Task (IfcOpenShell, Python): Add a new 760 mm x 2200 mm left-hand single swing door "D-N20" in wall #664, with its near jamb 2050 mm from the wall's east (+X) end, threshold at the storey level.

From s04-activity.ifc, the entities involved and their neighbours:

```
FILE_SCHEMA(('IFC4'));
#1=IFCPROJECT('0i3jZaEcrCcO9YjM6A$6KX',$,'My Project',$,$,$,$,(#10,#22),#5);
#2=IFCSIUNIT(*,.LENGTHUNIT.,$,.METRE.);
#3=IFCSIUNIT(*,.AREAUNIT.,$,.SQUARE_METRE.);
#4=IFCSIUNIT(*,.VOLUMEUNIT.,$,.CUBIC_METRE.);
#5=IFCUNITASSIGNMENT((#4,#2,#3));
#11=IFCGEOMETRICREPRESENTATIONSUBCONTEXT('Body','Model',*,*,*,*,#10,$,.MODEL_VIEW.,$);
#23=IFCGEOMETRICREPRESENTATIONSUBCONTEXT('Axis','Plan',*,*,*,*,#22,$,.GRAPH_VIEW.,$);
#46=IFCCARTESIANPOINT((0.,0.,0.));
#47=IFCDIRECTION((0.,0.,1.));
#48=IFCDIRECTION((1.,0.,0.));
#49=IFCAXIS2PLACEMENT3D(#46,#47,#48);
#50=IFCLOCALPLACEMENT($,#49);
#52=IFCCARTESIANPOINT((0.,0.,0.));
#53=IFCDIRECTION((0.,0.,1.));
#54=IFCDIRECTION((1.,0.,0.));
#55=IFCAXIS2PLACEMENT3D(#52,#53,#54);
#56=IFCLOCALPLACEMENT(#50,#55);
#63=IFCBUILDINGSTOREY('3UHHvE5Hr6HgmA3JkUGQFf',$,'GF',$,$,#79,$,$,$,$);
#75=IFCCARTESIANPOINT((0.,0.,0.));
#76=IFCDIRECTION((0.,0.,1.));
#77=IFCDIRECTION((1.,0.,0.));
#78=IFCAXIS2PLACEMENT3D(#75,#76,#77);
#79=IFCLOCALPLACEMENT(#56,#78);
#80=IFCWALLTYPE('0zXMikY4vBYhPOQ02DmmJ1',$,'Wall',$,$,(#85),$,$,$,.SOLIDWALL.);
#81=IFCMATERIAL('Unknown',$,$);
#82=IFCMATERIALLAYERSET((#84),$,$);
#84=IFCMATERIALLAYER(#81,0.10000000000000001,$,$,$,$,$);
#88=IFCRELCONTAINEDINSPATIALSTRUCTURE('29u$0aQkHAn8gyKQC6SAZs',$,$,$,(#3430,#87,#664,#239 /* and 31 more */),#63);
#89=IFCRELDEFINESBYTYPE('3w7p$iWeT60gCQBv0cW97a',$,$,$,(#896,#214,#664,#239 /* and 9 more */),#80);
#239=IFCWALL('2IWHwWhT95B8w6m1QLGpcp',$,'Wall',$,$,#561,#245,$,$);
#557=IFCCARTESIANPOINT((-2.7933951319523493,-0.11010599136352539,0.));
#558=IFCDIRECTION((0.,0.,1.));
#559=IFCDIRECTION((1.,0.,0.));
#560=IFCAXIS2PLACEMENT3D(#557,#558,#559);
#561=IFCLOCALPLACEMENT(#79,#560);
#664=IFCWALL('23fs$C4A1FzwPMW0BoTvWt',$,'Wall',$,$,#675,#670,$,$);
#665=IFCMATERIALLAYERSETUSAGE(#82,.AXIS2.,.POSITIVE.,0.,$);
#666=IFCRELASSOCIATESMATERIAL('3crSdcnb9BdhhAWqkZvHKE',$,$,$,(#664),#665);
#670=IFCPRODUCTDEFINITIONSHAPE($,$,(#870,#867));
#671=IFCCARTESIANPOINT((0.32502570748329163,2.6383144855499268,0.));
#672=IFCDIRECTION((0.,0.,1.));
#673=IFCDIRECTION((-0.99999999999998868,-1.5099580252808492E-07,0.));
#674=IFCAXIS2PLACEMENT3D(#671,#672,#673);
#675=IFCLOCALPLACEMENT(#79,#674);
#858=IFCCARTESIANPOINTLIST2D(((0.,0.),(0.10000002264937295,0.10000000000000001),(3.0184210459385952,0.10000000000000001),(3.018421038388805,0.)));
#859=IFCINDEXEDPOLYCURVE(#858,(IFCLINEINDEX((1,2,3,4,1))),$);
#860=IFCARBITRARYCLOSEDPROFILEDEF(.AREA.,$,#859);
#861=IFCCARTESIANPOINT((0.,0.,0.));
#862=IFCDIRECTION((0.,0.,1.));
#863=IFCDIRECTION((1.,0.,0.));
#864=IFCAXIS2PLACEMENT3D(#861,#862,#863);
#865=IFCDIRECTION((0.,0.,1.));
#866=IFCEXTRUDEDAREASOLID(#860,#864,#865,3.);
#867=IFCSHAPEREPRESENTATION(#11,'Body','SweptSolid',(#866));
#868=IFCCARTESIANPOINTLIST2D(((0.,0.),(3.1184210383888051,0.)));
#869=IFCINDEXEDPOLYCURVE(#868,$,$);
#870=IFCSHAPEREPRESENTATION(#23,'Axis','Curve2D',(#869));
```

```python
import numpy as np
import ifcopenshell
import ifcopenshell.api.feature
import ifcopenshell.api.geometry
import ifcopenshell.api.root
import ifcopenshell.api.spatial
import ifcopenshell.geom
import ifcopenshell.util.element
import ifcopenshell.util.placement
import ifcopenshell.util.representation
import ifcopenshell.util.shape
import ifcopenshell.util.unit

model = ifcopenshell.open("s04-activity.ifc")
unit_scale = ifcopenshell.util.unit.calculate_unit_scale(model)
settings = ifcopenshell.geom.settings()


def volume(element):
    """Net volume in cubic metres, openings subtracted."""
    shape = ifcopenshell.geom.create_shape(settings, element)
    return ifcopenshell.util.shape.get_volume(shape.geometry)


wall = model.by_guid("23fs$C4A1FzwPMW0BoTvWt")
storey = ifcopenshell.util.element.get_container(wall, ifc_class="IfcBuildingStorey")
context = ifcopenshell.util.representation.get_context(model, "Model", "Body", "MODEL_VIEW")
before = volume(wall)

width, height, from_end, sill = 0.76, 2.2, 2.05, 0.0  # metres

# The wall runs along its own X axis, and the end named is its -X end.
wall_shape = ifcopenshell.geom.create_shape(settings, wall)
x, y, z = ifcopenshell.util.shape.get_vertices(wall_shape.geometry).T
start = x.min() + from_end
face, thickness = float(y.min()), float(y.max() - y.min())
wall_matrix = ifcopenshell.util.placement.get_local_placement(wall.ObjectPlacement)
level = ifcopenshell.util.placement.get_local_placement(storey.ObjectPlacement)[2, 3]


def in_wall(x, y):
    """Placement at x, y metres in the wall's axes, at sill height."""
    matrix = wall_matrix.copy()
    matrix[:, 3] = wall_matrix @ np.array([x / unit_scale, y / unit_scale, 0.0, 1.0])
    matrix[2, 3] = level + sill / unit_scale
    return matrix


# Opening: a box that overshoots both wall faces by 50 mm.
opening = ifcopenshell.api.root.create_entity(model, ifc_class="IfcOpeningElement", predefined_type="OPENING")
box = ifcopenshell.api.geometry.add_wall_representation(
    model, context=context, length=width, height=height, thickness=thickness + 0.1
)
ifcopenshell.api.geometry.assign_representation(model, product=opening, representation=box)
ifcopenshell.api.geometry.edit_object_placement(model, product=opening, matrix=in_wall(start, face - 0.05), is_si=False)
ifcopenshell.api.feature.add_feature(model, feature=opening, element=wall)

door = ifcopenshell.api.root.create_entity(model, ifc_class="IfcDoor", name="D-N20", predefined_type="DOOR")
door.OverallWidth, door.OverallHeight = width / unit_scale, height / unit_scale
door.OperationType = "SINGLE_SWING_LEFT"
body = ifcopenshell.api.geometry.add_door_representation(
    model,
    context=context,
    overall_width=door.OverallWidth,
    overall_height=door.OverallHeight,
    operation_type="SINGLE_SWING_LEFT",
    lining_properties={"LiningDepth": thickness / unit_scale, "ThresholdDepth": thickness / unit_scale},
)
ifcopenshell.api.geometry.assign_representation(model, product=door, representation=body)
ifcopenshell.api.spatial.assign_container(model, products=[door], relating_structure=storey)
ifcopenshell.api.feature.add_filling(model, opening=opening, element=door)

# The lining spans the wall, so the door starts at the wall face.
ifcopenshell.api.geometry.edit_object_placement(model, product=door, matrix=in_wall(start, face), is_si=False)

after = volume(wall)

print(f"wall volume {before:.3f} -> {after:.3f} m3")

model.write("s04-activity-out.ifc")
```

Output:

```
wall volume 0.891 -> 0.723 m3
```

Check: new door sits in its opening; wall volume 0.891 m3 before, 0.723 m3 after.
